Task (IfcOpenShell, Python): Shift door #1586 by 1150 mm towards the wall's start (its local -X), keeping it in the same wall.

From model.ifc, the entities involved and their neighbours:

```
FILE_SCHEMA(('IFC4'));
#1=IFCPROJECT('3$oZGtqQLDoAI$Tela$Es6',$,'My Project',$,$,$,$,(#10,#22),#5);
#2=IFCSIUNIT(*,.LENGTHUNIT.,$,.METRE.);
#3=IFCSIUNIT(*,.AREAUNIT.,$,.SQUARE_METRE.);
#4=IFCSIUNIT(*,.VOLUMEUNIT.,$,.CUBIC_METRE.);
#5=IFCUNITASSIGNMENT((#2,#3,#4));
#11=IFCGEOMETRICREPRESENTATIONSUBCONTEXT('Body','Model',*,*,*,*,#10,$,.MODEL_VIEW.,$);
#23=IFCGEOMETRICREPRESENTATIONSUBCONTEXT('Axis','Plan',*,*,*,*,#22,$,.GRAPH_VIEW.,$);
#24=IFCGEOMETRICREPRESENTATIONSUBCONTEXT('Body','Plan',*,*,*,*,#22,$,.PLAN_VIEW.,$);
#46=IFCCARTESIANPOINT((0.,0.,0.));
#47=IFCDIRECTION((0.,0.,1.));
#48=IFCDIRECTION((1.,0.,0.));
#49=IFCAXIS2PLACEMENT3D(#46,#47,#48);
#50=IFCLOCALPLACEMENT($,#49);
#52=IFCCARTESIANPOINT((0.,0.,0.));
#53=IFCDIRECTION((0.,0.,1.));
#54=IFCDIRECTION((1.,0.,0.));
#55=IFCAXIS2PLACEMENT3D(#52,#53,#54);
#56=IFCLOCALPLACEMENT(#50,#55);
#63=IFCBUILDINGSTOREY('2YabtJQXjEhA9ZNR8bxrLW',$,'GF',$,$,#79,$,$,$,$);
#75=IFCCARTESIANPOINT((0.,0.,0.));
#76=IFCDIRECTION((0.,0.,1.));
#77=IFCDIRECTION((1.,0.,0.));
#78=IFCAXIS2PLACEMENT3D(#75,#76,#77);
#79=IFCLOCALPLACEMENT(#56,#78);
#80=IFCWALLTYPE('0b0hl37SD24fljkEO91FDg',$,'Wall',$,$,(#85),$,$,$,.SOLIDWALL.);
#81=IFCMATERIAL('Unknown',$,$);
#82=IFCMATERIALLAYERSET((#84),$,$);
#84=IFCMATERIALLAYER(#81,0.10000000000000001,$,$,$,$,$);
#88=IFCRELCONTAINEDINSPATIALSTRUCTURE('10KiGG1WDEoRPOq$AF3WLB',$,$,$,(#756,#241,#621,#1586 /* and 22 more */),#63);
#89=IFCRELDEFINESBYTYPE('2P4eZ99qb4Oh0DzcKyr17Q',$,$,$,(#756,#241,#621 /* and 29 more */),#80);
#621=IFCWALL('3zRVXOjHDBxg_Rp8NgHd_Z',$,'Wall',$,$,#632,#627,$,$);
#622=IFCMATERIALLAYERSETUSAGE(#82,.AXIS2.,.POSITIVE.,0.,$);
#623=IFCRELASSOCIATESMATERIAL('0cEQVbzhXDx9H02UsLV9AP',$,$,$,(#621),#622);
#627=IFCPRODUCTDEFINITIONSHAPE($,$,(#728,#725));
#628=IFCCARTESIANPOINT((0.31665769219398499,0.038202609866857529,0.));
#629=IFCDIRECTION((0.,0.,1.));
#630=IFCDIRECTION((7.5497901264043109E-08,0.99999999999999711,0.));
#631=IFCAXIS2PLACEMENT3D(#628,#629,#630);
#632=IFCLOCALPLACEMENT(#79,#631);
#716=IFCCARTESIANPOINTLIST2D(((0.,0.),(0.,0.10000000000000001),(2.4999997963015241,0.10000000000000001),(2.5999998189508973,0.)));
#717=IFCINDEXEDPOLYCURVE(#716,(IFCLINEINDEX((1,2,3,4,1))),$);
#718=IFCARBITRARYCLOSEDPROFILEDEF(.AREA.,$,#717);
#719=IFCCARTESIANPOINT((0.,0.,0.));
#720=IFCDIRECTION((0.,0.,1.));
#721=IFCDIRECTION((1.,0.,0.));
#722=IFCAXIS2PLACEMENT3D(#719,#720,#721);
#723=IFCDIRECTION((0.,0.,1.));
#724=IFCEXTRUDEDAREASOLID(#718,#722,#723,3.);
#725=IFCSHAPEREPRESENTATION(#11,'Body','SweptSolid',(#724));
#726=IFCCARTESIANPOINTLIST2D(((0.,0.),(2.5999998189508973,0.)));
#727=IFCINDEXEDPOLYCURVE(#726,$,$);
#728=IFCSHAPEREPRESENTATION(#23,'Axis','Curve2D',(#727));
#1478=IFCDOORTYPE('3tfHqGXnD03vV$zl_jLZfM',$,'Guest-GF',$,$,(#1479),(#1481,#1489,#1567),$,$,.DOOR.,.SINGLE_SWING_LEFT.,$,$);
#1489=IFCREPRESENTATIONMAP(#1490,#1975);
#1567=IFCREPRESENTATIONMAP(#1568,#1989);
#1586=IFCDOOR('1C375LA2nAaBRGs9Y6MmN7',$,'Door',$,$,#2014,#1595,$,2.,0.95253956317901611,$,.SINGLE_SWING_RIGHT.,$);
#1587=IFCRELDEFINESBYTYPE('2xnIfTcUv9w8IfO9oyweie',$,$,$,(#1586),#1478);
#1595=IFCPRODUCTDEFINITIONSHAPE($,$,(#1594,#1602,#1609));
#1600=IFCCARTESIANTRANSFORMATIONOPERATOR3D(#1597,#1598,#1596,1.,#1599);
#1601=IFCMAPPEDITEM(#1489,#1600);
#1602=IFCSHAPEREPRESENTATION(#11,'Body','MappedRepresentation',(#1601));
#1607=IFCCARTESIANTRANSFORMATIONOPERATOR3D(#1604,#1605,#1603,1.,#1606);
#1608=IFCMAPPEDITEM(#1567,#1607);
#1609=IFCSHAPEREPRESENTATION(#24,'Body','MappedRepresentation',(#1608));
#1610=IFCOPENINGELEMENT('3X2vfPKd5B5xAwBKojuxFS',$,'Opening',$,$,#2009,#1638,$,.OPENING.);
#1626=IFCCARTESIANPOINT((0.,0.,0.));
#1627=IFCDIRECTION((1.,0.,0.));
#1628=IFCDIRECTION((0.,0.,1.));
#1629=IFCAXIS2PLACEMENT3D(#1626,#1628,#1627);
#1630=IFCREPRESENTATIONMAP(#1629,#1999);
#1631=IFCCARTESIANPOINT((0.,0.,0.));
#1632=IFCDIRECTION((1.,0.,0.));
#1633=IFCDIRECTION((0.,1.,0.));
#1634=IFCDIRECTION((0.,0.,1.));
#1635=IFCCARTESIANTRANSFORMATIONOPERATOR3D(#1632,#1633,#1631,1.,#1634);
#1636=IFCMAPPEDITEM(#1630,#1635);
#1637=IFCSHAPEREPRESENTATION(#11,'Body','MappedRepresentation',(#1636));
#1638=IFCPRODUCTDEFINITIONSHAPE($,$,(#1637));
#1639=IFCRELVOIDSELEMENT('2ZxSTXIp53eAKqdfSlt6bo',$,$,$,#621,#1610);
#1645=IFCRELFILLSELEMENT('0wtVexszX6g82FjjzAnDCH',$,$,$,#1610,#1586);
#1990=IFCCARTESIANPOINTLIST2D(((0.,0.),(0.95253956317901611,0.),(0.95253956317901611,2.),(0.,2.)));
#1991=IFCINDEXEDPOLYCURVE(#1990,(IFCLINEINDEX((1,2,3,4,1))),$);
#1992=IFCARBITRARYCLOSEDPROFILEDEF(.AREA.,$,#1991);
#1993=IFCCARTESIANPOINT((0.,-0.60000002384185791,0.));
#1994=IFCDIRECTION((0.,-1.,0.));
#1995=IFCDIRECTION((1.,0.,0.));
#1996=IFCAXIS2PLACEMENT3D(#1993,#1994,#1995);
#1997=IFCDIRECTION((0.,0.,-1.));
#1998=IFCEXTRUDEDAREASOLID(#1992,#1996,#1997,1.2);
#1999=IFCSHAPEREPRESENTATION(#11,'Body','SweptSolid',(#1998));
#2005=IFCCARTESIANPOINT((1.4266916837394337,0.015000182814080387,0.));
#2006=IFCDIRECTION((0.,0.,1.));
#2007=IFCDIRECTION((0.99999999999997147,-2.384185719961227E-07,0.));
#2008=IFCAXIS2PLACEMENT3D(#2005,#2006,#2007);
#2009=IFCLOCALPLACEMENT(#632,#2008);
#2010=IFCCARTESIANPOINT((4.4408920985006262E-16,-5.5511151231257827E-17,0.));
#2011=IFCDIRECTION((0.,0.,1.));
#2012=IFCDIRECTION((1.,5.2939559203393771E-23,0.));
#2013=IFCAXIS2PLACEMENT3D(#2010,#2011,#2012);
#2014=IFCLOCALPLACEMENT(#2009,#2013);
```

```python
import ifcopenshell
import ifcopenshell.api.geometry
import ifcopenshell.util.placement
import ifcopenshell.util.unit

model = ifcopenshell.open("model.ifc")
unit_scale = ifcopenshell.util.unit.calculate_unit_scale(model)

door = model.by_guid("1C375LA2nAaBRGs9Y6MmN7")
opening = door.FillsVoids[0].RelatingOpeningElement
wall = opening.VoidsElements[0].RelatingBuildingElement

wall_matrix = ifcopenshell.util.placement.get_local_placement(wall.ObjectPlacement)
shift = wall_matrix[:3, 0] * -1.15 / unit_scale
before = ifcopenshell.util.placement.get_local_placement(door.ObjectPlacement)[:3, 3].copy()

# The door is placed relative to its opening, so it follows when the opening moves.
matrix = ifcopenshell.util.placement.get_local_placement(opening.ObjectPlacement)
matrix[:3, 3] += shift
ifcopenshell.api.geometry.edit_object_placement(
    model, product=opening, matrix=matrix, is_si=False, should_transform_children=True
)

after = ifcopenshell.util.placement.get_local_placement(door.ObjectPlacement)[:3, 3]
print("door moved by", (after - before).round(3) + 0.0)

model.write("model_edited.ifc")
```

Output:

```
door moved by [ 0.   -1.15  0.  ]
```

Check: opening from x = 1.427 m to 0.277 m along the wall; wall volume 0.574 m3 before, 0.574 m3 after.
